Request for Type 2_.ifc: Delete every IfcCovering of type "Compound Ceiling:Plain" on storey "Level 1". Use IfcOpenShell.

First a look at what the model holds.

```python
import ifcopenshell
import ifcopenshell.util.element

model = ifcopenshell.open("Type 2_.ifc")
print(model.schema)
storey = next(s for s in model.by_type("IfcBuildingStorey") if s.Name == "Level 1")
coverings = [e for e in ifcopenshell.util.element.get_decomposition(storey) if e.is_a("IfcCovering")]
seen = {}
for e in coverings:
    element_type = ifcopenshell.util.element.get_type(e)
    name = element_type.Name if element_type not in (None, e) else None
    seen[name] = seen.get(name, 0) + 1
for name, count in sorted(seen.items(), key=str):
    print(count, "x", name)
```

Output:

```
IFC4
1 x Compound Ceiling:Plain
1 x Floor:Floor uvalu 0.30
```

```python
import ifcopenshell
import ifcopenshell.api.root
import ifcopenshell.util.element

model = ifcopenshell.open("Type 2_.ifc")

storey = next(s for s in model.by_type("IfcBuildingStorey") if s.Name == "Level 1")
coverings = [e for e in ifcopenshell.util.element.get_decomposition(storey) if e.is_a("IfcCovering")]
targets = [e for e in coverings if (t := ifcopenshell.util.element.get_type(e)) not in (None, e) and t.Name == "Compound Ceiling:Plain"]

for e in targets:
    ifcopenshell.api.root.remove_product(model, product=e)
print(len(targets), "removed")

model.write("Type 2_-out.ifc")
```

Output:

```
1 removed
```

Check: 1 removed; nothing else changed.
